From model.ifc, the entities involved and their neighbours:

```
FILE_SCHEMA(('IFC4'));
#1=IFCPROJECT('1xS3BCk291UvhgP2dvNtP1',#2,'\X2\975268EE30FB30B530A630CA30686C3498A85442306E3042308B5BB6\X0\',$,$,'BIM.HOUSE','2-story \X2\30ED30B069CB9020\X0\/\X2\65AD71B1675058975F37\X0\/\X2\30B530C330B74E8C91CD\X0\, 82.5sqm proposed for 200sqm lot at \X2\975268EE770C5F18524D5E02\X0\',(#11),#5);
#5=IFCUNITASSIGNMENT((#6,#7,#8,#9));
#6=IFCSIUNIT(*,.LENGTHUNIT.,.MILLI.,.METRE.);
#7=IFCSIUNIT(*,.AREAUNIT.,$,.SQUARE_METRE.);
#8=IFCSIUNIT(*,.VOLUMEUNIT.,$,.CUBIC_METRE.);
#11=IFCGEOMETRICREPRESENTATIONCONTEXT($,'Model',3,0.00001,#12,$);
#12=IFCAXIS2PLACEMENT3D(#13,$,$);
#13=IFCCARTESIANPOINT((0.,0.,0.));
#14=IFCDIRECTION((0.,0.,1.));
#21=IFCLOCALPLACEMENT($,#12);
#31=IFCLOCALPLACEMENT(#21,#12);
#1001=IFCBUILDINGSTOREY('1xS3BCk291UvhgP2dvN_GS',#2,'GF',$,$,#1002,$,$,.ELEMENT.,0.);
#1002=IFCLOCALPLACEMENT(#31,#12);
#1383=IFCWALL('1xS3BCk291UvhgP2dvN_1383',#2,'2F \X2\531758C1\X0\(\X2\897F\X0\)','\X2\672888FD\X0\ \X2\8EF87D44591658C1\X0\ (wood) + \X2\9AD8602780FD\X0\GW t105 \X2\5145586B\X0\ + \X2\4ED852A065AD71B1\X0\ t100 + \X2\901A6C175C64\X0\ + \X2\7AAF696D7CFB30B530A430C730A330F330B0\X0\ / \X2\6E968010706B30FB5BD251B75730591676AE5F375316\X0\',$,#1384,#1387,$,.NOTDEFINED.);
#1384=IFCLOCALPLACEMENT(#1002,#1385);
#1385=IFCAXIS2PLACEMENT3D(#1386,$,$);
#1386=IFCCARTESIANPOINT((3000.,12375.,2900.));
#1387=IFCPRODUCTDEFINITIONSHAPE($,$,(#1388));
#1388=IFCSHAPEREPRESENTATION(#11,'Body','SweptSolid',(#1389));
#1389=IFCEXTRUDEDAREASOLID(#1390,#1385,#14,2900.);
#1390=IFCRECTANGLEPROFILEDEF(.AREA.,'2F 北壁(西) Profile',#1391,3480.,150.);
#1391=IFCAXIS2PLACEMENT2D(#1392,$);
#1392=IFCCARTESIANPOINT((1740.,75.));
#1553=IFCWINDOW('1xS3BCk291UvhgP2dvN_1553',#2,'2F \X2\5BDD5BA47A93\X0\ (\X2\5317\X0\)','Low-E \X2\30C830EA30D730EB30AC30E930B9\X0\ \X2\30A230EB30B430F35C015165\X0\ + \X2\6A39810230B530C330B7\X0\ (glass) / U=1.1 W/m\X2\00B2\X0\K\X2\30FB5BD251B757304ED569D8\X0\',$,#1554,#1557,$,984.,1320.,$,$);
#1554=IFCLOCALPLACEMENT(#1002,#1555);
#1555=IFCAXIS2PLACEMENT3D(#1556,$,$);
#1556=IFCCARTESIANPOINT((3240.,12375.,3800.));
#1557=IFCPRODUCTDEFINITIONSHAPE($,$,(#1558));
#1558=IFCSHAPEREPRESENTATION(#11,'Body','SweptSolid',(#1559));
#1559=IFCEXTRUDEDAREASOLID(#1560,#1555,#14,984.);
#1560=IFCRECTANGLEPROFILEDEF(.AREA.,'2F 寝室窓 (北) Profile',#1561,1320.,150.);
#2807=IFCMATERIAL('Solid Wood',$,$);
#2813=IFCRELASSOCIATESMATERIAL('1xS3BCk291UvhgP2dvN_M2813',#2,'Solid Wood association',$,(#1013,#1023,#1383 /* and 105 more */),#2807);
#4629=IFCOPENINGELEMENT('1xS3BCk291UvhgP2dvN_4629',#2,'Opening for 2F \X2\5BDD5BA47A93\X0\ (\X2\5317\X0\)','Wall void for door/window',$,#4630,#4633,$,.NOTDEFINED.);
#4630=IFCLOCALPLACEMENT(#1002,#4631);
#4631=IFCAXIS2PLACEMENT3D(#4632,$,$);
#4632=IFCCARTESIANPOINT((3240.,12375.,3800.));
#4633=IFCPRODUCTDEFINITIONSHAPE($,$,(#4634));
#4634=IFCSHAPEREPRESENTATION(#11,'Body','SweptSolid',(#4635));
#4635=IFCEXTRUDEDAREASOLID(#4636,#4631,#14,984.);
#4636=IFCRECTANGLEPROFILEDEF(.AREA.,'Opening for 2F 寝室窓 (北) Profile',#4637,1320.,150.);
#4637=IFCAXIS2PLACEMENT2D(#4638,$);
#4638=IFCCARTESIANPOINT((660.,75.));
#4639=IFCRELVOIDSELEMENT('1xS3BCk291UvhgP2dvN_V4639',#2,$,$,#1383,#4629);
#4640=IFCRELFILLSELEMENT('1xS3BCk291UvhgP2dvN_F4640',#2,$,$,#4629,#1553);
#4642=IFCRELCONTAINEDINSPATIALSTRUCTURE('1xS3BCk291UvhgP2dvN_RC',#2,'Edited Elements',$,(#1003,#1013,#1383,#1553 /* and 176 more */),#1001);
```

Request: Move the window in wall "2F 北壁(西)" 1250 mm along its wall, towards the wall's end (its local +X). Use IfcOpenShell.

```python
import ifcopenshell
import ifcopenshell.api.geometry
import ifcopenshell.util.placement
import ifcopenshell.util.unit

model = ifcopenshell.open("model.ifc")
unit_scale = ifcopenshell.util.unit.calculate_unit_scale(model)

window = model.by_guid("1xS3BCk291UvhgP2dvN_1553")
opening = window.FillsVoids[0].RelatingOpeningElement
wall = opening.VoidsElements[0].RelatingBuildingElement

wall_matrix = ifcopenshell.util.placement.get_local_placement(wall.ObjectPlacement)
shift = wall_matrix[:3, 0] * 1.25 / unit_scale
before = ifcopenshell.util.placement.get_local_placement(window.ObjectPlacement)[:3, 3].copy()

# The window is not placed relative to its opening, so move both.
for product in (opening, window):
    matrix = ifcopenshell.util.placement.get_local_placement(product.ObjectPlacement)
    matrix[:3, 3] += shift
    ifcopenshell.api.geometry.edit_object_placement(model, product=product, matrix=matrix, is_si=False)

after = ifcopenshell.util.placement.get_local_placement(window.ObjectPlacement)[:3, 3]
print("window moved by", (after - before).round(3) + 0.0)

model.write("model_updated.ifc")
```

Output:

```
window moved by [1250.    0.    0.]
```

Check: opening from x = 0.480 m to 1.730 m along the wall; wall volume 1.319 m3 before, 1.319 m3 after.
